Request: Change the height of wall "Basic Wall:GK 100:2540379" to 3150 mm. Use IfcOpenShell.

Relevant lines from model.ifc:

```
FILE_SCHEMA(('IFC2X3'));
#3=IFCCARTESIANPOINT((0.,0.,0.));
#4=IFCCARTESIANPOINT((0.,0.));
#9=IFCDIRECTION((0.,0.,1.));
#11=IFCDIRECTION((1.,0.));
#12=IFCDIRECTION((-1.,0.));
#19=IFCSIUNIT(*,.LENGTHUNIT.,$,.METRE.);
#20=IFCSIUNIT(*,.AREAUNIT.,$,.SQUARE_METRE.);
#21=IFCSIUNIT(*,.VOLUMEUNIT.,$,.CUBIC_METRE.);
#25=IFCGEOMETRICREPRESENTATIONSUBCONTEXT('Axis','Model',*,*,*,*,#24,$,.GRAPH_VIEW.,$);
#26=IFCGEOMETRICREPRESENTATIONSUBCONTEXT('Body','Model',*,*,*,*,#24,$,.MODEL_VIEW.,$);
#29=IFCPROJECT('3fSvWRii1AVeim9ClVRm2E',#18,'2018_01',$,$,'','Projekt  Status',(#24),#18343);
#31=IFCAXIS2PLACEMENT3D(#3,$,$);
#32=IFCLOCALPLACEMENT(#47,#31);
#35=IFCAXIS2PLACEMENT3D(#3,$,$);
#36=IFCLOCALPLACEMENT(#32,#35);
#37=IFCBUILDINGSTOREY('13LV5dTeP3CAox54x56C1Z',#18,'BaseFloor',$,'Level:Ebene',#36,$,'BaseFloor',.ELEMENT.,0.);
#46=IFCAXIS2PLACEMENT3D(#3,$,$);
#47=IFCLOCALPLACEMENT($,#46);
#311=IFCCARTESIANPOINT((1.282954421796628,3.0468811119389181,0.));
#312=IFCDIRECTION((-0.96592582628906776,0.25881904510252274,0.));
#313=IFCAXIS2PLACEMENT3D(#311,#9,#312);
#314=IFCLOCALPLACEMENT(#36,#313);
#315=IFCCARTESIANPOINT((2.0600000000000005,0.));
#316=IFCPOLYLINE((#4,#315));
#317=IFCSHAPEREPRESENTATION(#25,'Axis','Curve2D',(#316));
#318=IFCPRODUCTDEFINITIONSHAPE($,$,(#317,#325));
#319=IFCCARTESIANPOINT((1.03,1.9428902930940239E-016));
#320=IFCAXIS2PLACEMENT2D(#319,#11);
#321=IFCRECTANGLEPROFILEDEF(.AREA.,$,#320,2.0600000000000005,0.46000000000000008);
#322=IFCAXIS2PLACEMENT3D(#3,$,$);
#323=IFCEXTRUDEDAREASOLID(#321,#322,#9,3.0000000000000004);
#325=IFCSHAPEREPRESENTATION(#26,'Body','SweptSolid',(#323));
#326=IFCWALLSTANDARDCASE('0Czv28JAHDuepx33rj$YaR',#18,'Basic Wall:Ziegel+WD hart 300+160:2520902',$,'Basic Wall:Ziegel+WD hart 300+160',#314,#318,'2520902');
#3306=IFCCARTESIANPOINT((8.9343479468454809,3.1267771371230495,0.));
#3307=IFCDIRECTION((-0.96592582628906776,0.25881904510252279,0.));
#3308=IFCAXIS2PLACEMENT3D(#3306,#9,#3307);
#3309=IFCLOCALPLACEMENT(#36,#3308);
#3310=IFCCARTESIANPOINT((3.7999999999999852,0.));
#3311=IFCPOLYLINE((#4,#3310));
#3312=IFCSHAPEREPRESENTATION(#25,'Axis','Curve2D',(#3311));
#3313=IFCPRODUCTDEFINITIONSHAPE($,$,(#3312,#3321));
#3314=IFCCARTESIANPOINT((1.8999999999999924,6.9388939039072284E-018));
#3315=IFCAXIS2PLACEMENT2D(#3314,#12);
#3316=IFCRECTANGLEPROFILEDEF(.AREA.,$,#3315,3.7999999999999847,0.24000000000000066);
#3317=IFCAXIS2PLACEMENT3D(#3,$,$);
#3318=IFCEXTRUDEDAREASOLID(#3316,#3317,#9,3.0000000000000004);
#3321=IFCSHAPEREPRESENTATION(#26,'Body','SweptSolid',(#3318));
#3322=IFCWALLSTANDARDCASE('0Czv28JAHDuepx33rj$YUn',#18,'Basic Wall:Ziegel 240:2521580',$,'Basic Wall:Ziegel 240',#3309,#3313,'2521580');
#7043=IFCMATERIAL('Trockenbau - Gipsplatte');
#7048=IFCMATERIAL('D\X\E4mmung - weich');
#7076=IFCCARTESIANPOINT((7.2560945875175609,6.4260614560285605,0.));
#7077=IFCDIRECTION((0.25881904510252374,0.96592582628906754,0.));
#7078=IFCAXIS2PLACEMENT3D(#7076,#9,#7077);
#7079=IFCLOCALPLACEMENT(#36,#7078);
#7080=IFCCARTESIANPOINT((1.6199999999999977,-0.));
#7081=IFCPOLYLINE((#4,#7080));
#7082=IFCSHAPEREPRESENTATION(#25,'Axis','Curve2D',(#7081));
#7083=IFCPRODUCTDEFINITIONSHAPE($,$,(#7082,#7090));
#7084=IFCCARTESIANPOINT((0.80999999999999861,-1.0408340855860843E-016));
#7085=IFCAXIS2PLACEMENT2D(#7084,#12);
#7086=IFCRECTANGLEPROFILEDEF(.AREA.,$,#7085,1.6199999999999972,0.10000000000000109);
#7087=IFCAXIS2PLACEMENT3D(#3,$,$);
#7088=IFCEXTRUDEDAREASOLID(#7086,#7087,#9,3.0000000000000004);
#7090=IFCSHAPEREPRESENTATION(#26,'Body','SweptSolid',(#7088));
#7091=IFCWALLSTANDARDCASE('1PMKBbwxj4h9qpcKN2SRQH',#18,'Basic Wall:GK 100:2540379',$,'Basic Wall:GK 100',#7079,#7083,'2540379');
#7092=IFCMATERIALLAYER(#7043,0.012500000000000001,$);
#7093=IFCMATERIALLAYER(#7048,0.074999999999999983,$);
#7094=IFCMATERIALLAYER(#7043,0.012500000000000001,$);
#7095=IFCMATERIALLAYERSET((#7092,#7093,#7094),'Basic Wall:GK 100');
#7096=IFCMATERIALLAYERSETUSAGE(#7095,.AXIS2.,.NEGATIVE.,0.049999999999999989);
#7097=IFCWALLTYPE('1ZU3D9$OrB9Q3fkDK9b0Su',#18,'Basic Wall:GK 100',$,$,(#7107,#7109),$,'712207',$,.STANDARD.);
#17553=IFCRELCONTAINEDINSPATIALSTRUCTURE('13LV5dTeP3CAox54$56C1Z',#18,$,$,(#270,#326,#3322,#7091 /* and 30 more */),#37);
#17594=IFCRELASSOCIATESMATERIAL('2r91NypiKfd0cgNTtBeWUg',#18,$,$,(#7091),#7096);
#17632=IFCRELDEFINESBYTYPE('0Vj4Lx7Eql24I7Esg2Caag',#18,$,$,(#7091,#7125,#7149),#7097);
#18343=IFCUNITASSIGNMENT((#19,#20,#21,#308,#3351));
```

```python
import ifcopenshell
import ifcopenshell.geom
import ifcopenshell.util.representation
import ifcopenshell.util.shape

model = ifcopenshell.open("model.ifc")
settings = ifcopenshell.geom.settings()


def volume(element):
    """Net volume in cubic metres, openings subtracted."""
    shape = ifcopenshell.geom.create_shape(settings, element)
    return ifcopenshell.util.shape.get_volume(shape.geometry)


wall = model.by_guid("1PMKBbwxj4h9qpcKN2SRQH")
before = volume(wall)

body = ifcopenshell.util.representation.get_representation(wall, "Model", "Body")
solid = body.Items[0]
old_height = solid.Depth
solid.Depth = 3.15
after = volume(wall)

print(f"height {old_height:g} -> {solid.Depth:g}, volume {before:.3f} -> {after:.3f} m3")

model.write("model_rev.ifc")
```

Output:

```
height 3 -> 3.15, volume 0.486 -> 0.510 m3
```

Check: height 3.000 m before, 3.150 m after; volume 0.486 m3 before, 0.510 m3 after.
